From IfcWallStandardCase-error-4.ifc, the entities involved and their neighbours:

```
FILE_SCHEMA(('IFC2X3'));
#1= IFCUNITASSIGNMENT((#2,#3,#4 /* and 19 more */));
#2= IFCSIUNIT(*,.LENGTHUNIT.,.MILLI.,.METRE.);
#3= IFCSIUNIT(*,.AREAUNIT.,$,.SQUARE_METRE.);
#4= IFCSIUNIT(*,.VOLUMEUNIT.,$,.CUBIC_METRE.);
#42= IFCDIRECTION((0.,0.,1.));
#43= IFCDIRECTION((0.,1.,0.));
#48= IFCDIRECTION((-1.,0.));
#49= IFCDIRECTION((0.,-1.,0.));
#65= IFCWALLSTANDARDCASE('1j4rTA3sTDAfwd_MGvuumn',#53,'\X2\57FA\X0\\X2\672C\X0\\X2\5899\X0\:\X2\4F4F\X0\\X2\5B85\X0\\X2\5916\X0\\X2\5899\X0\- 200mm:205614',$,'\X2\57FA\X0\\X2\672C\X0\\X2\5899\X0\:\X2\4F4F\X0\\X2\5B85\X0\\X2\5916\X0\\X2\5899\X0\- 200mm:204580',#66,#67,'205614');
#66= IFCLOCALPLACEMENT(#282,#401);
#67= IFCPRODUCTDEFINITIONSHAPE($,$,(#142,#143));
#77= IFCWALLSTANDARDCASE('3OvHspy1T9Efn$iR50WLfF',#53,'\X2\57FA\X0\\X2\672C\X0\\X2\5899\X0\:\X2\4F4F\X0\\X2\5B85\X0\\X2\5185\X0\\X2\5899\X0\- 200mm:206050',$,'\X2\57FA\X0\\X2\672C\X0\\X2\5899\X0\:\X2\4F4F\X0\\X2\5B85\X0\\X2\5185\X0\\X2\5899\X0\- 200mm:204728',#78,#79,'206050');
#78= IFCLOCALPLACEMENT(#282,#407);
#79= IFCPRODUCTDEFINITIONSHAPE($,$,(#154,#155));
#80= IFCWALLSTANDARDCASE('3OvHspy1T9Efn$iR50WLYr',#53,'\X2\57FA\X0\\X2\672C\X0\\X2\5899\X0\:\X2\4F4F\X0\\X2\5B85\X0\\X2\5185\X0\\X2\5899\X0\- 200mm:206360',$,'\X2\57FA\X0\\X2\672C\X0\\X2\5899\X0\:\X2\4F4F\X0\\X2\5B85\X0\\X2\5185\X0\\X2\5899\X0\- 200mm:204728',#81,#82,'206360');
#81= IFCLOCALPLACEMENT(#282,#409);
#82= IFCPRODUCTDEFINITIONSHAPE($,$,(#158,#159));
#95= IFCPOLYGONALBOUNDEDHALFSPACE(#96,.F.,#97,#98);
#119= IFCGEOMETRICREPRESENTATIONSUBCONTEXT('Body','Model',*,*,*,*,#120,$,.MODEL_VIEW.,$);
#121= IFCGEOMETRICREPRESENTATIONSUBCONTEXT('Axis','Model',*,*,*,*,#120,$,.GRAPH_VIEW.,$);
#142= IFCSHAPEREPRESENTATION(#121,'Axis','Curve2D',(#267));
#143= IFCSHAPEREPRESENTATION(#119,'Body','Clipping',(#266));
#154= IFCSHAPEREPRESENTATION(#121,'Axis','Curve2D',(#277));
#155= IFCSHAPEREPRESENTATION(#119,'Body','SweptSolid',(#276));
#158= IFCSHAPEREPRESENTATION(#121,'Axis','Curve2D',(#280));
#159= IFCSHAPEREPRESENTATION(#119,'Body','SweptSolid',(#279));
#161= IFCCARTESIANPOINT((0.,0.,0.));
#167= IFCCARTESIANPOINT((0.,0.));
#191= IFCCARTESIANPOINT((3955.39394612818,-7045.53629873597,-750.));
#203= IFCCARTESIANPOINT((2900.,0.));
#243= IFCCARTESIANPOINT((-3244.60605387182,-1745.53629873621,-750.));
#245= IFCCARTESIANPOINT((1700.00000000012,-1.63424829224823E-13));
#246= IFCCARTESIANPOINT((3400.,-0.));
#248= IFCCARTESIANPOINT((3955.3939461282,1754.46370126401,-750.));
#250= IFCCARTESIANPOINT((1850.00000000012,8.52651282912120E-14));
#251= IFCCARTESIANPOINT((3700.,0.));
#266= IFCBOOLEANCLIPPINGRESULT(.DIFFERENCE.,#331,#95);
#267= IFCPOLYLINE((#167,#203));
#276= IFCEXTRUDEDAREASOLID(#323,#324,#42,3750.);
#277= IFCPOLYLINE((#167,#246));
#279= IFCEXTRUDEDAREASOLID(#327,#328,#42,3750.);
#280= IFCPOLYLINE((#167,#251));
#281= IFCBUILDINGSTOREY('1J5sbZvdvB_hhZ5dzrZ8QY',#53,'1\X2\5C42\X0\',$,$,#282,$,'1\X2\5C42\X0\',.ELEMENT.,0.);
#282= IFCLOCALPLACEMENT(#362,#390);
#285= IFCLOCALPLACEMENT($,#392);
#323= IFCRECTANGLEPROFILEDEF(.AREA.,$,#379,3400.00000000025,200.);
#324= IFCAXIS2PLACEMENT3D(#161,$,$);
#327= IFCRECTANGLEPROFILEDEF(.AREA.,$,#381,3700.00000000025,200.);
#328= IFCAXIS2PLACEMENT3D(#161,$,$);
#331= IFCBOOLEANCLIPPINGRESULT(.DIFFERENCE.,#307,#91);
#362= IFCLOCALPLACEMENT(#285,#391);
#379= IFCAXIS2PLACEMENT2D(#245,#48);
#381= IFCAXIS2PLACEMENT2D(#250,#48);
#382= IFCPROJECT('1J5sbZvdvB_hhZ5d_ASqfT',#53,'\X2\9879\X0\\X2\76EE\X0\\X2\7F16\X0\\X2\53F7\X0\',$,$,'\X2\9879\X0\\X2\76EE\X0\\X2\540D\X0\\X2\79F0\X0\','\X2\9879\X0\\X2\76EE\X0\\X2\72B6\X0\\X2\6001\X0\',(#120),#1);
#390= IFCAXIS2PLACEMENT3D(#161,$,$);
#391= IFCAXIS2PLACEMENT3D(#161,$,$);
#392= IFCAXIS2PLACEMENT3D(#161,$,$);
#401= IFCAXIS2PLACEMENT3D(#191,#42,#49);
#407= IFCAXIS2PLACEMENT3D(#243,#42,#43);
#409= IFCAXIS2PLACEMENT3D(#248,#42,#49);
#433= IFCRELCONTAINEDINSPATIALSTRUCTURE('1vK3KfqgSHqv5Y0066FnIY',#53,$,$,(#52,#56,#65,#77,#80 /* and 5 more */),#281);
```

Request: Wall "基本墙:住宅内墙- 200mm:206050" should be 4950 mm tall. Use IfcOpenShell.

```python
import ifcopenshell
import ifcopenshell.geom
import ifcopenshell.util.representation
import ifcopenshell.util.shape
import ifcopenshell.util.unit

model = ifcopenshell.open("IfcWallStandardCase-error-4.ifc")
unit_scale = ifcopenshell.util.unit.calculate_unit_scale(model)
settings = ifcopenshell.geom.settings()


def volume(element):
    """Net volume in cubic metres, openings subtracted."""
    shape = ifcopenshell.geom.create_shape(settings, element)
    return ifcopenshell.util.shape.get_volume(shape.geometry)


wall = model.by_guid("3OvHspy1T9Efn$iR50WLfF")
before = volume(wall)

body = ifcopenshell.util.representation.get_representation(wall, "Model", "Body")
solid = body.Items[0]
old_height = solid.Depth
solid.Depth = 4.95 / unit_scale
after = volume(wall)

print(f"height {old_height:g} -> {solid.Depth:g}, volume {before:.3f} -> {after:.3f} m3")

model.write("IfcWallStandardCase-error-4_edited.ifc")
```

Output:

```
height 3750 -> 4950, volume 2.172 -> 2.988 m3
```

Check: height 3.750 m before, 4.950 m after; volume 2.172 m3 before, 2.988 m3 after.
